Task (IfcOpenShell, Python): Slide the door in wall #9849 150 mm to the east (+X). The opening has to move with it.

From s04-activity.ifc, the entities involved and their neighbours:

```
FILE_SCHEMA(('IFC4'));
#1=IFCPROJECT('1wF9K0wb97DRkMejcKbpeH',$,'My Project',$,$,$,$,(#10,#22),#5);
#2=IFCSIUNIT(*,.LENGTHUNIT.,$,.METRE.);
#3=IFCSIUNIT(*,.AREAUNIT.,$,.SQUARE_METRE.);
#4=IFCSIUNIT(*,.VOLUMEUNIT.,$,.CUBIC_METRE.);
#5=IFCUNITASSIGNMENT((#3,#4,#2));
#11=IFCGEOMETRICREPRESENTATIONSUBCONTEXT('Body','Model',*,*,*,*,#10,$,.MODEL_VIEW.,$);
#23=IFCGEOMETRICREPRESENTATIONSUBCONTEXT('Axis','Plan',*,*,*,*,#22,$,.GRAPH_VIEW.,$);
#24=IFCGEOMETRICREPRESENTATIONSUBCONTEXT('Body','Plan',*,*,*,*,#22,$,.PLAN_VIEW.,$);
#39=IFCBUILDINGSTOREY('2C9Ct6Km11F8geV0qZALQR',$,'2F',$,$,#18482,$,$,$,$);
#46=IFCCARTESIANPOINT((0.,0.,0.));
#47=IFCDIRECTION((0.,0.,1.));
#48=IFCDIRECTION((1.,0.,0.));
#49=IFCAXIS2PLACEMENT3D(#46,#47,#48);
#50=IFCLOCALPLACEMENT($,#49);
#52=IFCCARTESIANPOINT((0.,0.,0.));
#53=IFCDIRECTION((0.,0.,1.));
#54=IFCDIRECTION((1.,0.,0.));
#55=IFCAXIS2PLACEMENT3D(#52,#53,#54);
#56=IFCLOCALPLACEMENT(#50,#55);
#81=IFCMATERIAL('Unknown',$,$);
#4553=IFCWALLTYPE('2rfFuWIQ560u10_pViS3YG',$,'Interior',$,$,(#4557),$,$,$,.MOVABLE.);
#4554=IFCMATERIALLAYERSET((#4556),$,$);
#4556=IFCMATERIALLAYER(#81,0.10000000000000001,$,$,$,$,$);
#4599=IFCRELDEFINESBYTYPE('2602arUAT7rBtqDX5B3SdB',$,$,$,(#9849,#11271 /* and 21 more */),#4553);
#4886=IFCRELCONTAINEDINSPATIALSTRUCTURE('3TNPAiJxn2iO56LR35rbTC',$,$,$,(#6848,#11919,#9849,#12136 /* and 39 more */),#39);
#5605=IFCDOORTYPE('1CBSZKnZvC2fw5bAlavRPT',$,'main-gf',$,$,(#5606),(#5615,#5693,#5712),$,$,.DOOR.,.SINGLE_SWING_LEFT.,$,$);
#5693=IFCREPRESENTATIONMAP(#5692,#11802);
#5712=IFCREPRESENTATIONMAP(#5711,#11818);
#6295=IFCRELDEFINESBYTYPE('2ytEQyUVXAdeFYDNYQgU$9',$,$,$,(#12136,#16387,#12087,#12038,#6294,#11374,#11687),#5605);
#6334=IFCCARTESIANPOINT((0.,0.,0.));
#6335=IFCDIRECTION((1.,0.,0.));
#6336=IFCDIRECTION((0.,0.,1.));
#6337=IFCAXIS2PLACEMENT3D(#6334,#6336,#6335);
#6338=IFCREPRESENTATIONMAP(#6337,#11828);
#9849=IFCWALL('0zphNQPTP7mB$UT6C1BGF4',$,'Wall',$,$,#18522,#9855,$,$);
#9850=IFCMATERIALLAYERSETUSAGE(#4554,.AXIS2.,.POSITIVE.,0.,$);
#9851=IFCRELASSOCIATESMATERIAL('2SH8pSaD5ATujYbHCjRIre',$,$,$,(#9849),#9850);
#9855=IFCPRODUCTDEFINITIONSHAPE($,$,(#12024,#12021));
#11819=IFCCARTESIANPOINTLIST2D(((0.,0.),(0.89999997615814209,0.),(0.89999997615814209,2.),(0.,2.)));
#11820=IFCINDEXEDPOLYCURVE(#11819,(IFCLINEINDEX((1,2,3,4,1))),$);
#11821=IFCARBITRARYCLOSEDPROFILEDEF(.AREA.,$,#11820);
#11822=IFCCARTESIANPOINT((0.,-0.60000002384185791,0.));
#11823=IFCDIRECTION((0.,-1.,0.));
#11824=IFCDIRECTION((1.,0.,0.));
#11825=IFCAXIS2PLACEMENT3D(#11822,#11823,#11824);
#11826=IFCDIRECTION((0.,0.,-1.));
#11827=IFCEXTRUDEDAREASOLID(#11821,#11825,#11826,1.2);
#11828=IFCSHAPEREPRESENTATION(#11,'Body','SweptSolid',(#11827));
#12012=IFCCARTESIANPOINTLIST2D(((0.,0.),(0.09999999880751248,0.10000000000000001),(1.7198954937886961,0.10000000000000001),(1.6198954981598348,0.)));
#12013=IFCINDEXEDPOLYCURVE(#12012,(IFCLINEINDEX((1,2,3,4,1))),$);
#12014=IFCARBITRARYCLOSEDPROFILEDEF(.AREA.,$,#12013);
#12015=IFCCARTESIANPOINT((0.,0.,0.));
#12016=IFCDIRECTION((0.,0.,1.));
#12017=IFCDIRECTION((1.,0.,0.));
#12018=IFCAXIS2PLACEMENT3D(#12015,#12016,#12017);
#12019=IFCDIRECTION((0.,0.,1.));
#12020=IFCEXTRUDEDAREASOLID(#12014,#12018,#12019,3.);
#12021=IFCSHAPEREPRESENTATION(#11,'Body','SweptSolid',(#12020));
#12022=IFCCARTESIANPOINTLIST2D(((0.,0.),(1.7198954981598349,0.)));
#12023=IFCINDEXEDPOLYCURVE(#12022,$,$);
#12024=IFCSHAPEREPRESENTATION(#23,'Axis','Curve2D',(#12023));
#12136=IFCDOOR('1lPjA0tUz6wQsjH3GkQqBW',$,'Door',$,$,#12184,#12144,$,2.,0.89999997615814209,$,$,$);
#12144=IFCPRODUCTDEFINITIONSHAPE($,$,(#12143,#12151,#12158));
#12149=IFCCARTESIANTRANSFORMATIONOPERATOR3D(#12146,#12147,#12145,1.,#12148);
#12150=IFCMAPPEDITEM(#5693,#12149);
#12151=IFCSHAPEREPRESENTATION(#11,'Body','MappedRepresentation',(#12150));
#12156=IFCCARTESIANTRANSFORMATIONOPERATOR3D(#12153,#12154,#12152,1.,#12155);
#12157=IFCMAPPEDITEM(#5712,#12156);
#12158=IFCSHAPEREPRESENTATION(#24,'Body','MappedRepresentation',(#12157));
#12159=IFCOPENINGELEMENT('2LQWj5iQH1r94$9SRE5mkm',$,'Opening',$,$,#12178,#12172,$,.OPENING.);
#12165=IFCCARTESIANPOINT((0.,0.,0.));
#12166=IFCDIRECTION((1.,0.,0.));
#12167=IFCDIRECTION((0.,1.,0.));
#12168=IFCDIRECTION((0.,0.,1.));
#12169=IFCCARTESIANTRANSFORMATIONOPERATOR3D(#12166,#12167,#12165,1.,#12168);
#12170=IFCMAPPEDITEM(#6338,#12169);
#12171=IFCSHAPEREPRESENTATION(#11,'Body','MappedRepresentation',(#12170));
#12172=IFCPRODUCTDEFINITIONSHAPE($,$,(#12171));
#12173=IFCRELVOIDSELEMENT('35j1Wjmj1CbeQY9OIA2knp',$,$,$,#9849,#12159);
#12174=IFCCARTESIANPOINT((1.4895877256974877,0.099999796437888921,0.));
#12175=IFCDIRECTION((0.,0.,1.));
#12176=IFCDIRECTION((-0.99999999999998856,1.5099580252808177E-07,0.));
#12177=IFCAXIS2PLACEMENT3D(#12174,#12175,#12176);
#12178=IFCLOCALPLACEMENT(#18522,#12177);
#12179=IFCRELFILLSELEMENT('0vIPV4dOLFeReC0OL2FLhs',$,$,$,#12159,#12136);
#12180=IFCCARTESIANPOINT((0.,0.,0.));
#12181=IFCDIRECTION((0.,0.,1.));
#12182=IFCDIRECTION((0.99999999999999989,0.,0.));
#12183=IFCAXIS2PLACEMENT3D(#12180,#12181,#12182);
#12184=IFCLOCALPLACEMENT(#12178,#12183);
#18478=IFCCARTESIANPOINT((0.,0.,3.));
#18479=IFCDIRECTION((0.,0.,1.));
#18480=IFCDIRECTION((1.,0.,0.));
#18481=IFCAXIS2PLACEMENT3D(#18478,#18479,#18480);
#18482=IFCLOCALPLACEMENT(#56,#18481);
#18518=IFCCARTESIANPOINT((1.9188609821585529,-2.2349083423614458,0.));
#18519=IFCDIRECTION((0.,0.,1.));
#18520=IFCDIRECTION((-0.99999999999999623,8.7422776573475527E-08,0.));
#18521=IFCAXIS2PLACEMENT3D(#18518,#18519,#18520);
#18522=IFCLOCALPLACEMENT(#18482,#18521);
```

```python
import ifcopenshell
import ifcopenshell.api.geometry
import ifcopenshell.util.placement

model = ifcopenshell.open("s04-activity.ifc")

door = model.by_guid("1lPjA0tUz6wQsjH3GkQqBW")
opening = door.FillsVoids[0].RelatingOpeningElement
wall = opening.VoidsElements[0].RelatingBuildingElement

wall_matrix = ifcopenshell.util.placement.get_local_placement(wall.ObjectPlacement)
shift = wall_matrix[:3, 0] * -0.15
before = ifcopenshell.util.placement.get_local_placement(door.ObjectPlacement)[:3, 3].copy()

# The door is placed relative to its opening, so it follows when the opening moves.
matrix = ifcopenshell.util.placement.get_local_placement(opening.ObjectPlacement)
matrix[:3, 3] += shift
ifcopenshell.api.geometry.edit_object_placement(
    model, product=opening, matrix=matrix, is_si=False, should_transform_children=True
)

after = ifcopenshell.util.placement.get_local_placement(door.ObjectPlacement)[:3, 3]
print("door moved by", (after - before).round(3) + 0.0)

model.write("s04-activity-out.ifc")
```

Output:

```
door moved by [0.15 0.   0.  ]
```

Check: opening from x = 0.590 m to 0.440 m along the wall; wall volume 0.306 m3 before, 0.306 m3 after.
